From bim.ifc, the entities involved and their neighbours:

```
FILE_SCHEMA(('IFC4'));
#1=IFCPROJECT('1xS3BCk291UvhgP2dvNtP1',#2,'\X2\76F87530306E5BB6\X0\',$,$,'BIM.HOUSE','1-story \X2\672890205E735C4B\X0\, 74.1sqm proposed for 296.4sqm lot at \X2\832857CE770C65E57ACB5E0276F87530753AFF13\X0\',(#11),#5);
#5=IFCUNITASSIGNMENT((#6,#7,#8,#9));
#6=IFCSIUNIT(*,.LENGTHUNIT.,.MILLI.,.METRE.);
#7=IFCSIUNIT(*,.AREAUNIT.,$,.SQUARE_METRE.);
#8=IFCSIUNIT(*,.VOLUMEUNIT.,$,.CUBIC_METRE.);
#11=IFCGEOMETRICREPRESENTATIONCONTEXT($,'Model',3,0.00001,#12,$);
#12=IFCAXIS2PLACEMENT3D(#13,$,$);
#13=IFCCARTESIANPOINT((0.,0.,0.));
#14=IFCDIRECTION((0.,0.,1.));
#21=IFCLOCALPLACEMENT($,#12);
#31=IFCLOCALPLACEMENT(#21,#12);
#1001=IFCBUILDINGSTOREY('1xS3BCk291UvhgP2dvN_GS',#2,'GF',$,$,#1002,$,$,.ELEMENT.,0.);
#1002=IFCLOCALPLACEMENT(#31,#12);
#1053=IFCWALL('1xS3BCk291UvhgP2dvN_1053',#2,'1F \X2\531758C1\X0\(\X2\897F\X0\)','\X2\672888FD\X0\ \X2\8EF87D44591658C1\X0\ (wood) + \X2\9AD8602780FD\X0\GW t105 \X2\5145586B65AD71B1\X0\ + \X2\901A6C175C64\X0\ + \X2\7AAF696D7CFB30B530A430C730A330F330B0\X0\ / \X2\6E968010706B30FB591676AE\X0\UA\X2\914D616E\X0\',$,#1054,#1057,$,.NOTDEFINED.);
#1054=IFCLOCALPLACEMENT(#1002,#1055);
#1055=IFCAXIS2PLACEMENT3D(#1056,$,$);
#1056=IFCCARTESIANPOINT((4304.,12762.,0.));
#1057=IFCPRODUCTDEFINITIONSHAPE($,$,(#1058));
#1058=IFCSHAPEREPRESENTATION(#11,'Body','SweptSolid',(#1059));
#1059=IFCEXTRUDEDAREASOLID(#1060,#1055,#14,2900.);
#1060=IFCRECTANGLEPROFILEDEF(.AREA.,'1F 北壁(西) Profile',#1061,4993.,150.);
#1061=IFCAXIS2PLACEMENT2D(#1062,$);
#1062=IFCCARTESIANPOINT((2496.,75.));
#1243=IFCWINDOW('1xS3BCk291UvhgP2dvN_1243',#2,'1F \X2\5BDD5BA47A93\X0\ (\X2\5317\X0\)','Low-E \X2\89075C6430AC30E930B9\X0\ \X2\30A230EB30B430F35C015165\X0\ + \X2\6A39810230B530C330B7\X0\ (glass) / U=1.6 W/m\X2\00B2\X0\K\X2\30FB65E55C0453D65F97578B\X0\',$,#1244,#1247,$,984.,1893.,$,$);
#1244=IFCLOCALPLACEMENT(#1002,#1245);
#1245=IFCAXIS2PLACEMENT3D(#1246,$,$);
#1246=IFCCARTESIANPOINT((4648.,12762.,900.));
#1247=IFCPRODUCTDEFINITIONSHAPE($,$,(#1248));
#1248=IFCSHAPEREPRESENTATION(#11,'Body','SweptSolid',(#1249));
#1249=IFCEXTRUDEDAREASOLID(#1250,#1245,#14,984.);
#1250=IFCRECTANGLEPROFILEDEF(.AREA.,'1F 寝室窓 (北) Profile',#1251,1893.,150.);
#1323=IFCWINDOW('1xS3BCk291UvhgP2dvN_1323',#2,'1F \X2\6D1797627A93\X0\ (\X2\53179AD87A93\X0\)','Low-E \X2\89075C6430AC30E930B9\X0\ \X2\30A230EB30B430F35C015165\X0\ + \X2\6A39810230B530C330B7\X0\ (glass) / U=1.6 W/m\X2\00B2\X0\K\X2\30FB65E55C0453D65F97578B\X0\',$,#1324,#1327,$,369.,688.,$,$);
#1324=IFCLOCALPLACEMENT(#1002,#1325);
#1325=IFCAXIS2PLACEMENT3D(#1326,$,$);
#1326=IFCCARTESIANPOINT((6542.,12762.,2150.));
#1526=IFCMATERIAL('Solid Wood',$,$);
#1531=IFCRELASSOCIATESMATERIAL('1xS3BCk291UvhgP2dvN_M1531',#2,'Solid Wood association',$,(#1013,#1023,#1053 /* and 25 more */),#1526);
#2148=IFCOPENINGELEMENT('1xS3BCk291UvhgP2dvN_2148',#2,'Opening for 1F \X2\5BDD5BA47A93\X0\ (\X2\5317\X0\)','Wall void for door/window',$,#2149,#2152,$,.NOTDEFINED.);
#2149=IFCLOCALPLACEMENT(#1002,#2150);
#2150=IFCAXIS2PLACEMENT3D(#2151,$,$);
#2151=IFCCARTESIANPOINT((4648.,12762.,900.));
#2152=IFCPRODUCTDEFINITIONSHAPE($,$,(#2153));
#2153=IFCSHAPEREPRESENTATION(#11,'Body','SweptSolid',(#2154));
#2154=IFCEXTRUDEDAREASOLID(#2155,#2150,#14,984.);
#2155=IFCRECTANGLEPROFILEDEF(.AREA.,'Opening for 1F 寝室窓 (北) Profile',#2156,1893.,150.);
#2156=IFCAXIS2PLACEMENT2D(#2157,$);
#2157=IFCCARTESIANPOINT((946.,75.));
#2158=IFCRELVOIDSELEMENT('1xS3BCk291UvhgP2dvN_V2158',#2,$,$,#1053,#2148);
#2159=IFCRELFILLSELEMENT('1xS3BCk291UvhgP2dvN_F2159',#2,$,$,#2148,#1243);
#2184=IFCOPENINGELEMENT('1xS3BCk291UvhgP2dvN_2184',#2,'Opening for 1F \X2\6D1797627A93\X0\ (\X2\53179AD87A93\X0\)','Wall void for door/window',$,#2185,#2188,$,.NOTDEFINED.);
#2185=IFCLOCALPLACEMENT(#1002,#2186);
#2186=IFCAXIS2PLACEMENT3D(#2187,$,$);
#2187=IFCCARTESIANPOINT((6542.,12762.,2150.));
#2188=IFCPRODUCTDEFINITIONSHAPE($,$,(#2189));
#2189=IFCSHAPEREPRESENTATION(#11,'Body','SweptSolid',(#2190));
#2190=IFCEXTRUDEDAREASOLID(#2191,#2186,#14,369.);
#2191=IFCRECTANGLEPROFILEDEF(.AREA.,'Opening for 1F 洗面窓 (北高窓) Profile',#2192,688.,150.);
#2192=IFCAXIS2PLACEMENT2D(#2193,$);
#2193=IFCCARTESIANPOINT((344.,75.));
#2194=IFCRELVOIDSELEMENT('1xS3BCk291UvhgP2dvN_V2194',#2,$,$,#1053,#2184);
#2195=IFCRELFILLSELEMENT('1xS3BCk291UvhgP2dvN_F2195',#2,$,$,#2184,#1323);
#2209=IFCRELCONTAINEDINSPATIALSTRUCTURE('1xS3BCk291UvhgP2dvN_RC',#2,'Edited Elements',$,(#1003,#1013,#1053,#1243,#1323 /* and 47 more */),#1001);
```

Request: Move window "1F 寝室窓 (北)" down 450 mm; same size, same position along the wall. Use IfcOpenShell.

```python
import numpy as np
import ifcopenshell
import ifcopenshell.api.geometry
import ifcopenshell.util.placement
import ifcopenshell.util.unit

model = ifcopenshell.open("bim.ifc")
unit_scale = ifcopenshell.util.unit.calculate_unit_scale(model)

window = model.by_guid("1xS3BCk291UvhgP2dvN_1243")
opening = window.FillsVoids[0].RelatingOpeningElement
dz = -0.45 / unit_scale

shift = np.array([0.0, 0.0, dz])
# The window is not placed relative to its opening, so move both.
for product in (opening, window):
    matrix = ifcopenshell.util.placement.get_local_placement(product.ObjectPlacement)
    matrix[:3, 3] += shift
    ifcopenshell.api.geometry.edit_object_placement(model, product=product, matrix=matrix, is_si=False)

print(f"moved by {dz * unit_scale:+.3f} m")

model.write("bim_v2.ifc")
```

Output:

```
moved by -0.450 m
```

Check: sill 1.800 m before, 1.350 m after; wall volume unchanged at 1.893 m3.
